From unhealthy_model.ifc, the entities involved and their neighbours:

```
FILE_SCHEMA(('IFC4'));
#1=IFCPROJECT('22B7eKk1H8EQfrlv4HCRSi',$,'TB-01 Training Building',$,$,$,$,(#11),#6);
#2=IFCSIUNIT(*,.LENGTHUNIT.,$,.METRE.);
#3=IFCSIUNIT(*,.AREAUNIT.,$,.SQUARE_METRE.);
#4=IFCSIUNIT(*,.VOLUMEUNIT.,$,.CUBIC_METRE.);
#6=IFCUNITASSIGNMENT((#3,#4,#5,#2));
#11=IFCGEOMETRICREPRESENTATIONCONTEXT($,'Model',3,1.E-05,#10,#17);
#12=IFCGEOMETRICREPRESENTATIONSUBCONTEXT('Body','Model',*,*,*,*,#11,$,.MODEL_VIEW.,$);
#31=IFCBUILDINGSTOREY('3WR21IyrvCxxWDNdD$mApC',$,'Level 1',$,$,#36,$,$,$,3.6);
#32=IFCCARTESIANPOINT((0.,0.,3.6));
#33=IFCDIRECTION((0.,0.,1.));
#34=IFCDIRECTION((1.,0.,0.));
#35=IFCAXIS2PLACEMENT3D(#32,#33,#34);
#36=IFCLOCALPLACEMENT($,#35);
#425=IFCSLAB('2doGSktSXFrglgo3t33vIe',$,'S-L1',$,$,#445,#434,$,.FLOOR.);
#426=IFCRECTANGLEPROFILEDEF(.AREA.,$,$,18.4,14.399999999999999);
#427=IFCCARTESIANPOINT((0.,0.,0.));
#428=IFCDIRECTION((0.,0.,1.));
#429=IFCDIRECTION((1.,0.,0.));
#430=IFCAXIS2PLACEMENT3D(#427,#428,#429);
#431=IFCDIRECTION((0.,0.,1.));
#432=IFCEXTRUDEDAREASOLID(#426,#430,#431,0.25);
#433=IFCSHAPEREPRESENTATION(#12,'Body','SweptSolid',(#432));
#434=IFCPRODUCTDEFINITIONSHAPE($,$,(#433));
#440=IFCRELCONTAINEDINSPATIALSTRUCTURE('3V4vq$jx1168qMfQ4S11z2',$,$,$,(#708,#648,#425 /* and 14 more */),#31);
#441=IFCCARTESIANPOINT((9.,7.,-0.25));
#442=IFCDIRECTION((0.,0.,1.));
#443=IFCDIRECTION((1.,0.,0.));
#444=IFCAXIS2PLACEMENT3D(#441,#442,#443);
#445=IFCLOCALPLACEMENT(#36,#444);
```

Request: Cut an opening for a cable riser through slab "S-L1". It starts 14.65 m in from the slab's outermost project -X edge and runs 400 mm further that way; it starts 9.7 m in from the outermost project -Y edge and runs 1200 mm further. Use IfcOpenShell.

```python
import numpy as np
import ifcopenshell
import ifcopenshell.api.feature
import ifcopenshell.api.geometry
import ifcopenshell.api.root
import ifcopenshell.geom
import ifcopenshell.util.placement
import ifcopenshell.util.representation
import ifcopenshell.util.shape
import ifcopenshell.util.unit

model = ifcopenshell.open("unhealthy_model.ifc")
unit_scale = ifcopenshell.util.unit.calculate_unit_scale(model)
settings = ifcopenshell.geom.settings()


def volume(element):
    """Net volume in cubic metres, openings subtracted."""
    shape = ifcopenshell.geom.create_shape(settings, element)
    return ifcopenshell.util.shape.get_volume(shape.geometry)


slab = model.by_id(425)
before = volume(slab)

# Extent in the slab's own axes, in metres. The edges named are its -X and -Y sides.
slab_shape = ifcopenshell.geom.create_shape(settings, slab)
vertices = ifcopenshell.util.shape.get_vertices(slab_shape.geometry)
x_min, y_min, bottom = vertices.min(axis=0)
top = vertices[:, 2].max()

opening = ifcopenshell.api.root.create_entity(model, ifc_class="IfcOpeningElement", name="Cable riser opening", predefined_type="OPENING")
context = ifcopenshell.util.representation.get_context(model, "Model", "Body", "MODEL_VIEW")
width, depth = 0.4, 1.2
outline = [(0.0, 0.0), (width, 0.0), (width, depth), (0.0, depth), (0.0, 0.0)]
# Overshoot both faces by 50 mm so the cut is clean.
shape = ifcopenshell.api.geometry.add_slab_representation(
    model, context=context, depth=top - bottom + 0.1, polyline=outline
)
ifcopenshell.api.geometry.assign_representation(model, product=opening, representation=shape)

matrix = ifcopenshell.util.placement.get_local_placement(slab.ObjectPlacement)
matrix[:, 3] = matrix @ np.append(np.array([x_min + 14.65, y_min + 9.7, bottom - 0.05]) / unit_scale, 1.0)
ifcopenshell.api.geometry.edit_object_placement(model, product=opening, matrix=matrix, is_si=False)
ifcopenshell.api.feature.add_feature(model, feature=opening, element=slab)

after = volume(slab)

print(f"slab volume {before:.3f} -> {after:.3f} m3")

model.write("unhealthy_model_updated.ifc")
```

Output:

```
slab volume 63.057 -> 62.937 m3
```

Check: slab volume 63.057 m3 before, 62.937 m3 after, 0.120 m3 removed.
